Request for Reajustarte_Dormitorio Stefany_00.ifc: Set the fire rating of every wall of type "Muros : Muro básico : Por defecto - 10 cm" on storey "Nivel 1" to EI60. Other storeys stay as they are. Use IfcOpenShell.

First a look at what the model holds.

```python
import ifcopenshell
import ifcopenshell.util.element

model = ifcopenshell.open("Reajustarte_Dormitorio Stefany_00.ifc")
print(model.schema)
storey = next(s for s in model.by_type("IfcBuildingStorey") if s.Name == "Nivel 1")
walls = [e for e in ifcopenshell.util.element.get_decomposition(storey) if e.is_a("IfcWall")]
seen = {}
for e in walls:
    element_type = ifcopenshell.util.element.get_type(e)
    key = (element_type.Name if element_type != e and element_type else None, ifcopenshell.util.element.get_pset(e, "Pset_WallCommon", "FireRating"))
    seen[key] = seen.get(key, 0) + 1
for (name, value), count in sorted(seen.items(), key=str):
    print(count, "x", name, "|", value)
```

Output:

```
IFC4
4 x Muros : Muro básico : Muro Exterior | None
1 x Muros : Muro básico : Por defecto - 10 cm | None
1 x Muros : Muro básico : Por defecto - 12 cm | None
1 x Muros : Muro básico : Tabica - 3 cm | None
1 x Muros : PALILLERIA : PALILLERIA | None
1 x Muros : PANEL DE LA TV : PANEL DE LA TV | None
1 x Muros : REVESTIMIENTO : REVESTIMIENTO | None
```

```python
import ifcopenshell
import ifcopenshell.api.pset
import ifcopenshell.util.element

model = ifcopenshell.open("Reajustarte_Dormitorio Stefany_00.ifc")

storey = next(s for s in model.by_type("IfcBuildingStorey") if s.Name == "Nivel 1")
walls = [e for e in ifcopenshell.util.element.get_decomposition(storey) if e.is_a("IfcWall")]

count = 0
for e in walls:
    element_type = ifcopenshell.util.element.get_type(e)
    if element_type in (None, e) or element_type.Name != "Muros : Muro básico : Por defecto - 10 cm":
        continue
    # add_pset returns the element's existing set when there is one.
    pset = ifcopenshell.api.pset.add_pset(model, product=e, name="Pset_WallCommon")
    ifcopenshell.api.pset.edit_pset(model, pset=pset, properties={"FireRating": "EI60"})
    count += 1

print(count, "walls updated")

model.write("Reajustarte_Dormitorio Stefany_00_updated.ifc")
```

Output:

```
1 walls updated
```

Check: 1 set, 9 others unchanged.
